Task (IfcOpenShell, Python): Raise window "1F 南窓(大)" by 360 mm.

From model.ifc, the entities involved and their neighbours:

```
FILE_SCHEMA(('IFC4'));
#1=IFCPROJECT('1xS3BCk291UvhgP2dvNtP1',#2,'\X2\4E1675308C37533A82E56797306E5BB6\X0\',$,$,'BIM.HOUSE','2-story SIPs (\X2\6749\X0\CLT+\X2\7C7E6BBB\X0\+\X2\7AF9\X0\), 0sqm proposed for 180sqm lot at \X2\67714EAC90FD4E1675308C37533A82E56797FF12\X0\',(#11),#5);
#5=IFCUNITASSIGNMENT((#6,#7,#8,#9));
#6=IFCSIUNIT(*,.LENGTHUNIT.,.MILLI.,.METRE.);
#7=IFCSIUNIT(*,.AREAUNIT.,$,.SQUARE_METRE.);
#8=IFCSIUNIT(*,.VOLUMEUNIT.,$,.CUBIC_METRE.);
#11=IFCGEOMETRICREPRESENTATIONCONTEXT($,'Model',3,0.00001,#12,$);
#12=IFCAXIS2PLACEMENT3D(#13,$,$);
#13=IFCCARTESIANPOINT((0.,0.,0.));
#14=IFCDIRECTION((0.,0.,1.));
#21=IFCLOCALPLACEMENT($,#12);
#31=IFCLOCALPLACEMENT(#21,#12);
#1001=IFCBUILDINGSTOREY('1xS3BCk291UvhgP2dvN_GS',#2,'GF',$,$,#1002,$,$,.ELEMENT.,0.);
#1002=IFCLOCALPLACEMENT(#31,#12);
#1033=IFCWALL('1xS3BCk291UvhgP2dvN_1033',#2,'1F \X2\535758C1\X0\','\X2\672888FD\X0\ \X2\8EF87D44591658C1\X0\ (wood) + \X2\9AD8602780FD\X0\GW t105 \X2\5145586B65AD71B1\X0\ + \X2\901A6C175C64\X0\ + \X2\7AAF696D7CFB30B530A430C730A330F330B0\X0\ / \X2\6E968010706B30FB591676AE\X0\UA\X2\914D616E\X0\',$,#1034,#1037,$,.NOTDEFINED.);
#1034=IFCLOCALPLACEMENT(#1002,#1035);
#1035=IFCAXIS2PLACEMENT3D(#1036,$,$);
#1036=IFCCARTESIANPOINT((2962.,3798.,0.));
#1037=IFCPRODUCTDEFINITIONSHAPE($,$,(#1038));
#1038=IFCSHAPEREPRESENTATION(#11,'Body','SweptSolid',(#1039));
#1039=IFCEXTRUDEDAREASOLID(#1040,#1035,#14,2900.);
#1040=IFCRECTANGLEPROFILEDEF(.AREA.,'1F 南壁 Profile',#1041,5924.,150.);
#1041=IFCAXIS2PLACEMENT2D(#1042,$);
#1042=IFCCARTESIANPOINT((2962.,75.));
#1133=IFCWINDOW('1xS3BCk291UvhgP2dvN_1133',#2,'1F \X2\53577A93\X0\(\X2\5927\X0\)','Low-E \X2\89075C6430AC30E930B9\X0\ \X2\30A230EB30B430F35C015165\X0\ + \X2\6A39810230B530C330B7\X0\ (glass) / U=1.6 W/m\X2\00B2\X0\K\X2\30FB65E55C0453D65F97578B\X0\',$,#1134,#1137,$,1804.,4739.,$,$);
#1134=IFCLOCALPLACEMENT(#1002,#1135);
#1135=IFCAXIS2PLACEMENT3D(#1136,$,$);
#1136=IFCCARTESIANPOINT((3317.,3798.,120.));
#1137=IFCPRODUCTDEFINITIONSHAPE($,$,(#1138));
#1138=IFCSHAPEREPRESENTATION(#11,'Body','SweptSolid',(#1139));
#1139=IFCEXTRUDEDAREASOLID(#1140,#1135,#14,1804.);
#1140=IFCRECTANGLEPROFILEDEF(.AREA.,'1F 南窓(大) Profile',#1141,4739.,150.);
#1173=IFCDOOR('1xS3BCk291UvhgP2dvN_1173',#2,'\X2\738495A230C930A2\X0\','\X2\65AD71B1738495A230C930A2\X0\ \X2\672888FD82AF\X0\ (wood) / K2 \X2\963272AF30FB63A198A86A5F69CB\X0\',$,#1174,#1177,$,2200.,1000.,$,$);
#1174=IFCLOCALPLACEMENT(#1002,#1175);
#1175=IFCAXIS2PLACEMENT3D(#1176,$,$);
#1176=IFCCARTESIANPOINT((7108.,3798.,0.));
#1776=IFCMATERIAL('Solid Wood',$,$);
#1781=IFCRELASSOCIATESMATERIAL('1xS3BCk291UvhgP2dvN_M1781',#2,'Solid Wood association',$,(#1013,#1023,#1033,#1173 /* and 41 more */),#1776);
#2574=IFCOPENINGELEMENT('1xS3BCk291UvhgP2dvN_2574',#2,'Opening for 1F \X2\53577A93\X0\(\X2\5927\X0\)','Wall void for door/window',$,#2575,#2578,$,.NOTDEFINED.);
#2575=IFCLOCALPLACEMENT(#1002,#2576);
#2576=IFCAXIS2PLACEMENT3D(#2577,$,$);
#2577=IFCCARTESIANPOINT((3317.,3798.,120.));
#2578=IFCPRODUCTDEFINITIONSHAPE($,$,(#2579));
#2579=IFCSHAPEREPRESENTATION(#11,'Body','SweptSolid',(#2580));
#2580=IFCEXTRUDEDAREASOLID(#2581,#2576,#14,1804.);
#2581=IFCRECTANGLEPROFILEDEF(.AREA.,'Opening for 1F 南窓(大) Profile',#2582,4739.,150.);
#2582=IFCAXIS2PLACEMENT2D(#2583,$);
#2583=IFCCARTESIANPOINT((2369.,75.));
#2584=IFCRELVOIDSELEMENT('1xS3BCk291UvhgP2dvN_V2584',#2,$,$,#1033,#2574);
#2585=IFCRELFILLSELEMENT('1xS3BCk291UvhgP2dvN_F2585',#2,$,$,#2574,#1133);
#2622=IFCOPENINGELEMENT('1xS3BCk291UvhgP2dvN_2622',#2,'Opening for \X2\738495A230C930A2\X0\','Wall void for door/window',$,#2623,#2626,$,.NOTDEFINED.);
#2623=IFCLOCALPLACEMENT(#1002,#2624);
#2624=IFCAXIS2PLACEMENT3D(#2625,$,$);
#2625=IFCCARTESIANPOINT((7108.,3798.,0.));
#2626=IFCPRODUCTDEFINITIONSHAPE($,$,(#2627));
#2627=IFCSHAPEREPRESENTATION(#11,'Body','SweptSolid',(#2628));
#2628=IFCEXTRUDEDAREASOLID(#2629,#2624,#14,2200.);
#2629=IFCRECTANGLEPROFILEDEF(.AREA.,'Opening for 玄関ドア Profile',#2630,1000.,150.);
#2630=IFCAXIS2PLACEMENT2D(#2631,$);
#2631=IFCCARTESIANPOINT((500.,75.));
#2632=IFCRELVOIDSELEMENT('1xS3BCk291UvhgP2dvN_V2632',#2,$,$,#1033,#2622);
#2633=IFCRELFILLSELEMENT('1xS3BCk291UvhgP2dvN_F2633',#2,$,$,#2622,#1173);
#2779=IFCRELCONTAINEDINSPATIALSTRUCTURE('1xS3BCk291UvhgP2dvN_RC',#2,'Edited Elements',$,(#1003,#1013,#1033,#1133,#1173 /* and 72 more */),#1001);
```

```python
import numpy as np
import ifcopenshell
import ifcopenshell.api.geometry
import ifcopenshell.util.placement
import ifcopenshell.util.unit

model = ifcopenshell.open("model.ifc")
unit_scale = ifcopenshell.util.unit.calculate_unit_scale(model)

window = model.by_guid("1xS3BCk291UvhgP2dvN_1133")
opening = window.FillsVoids[0].RelatingOpeningElement
dz = 0.36 / unit_scale

shift = np.array([0.0, 0.0, dz])
# The window is not placed relative to its opening, so move both.
for product in (opening, window):
    matrix = ifcopenshell.util.placement.get_local_placement(product.ObjectPlacement)
    matrix[:3, 3] += shift
    ifcopenshell.api.geometry.edit_object_placement(model, product=product, matrix=matrix, is_si=False)

print(f"moved by {dz * unit_scale:+.3f} m")

model.write("model_edited.ifc")
```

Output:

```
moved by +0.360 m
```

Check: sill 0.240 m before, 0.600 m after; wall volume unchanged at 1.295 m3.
